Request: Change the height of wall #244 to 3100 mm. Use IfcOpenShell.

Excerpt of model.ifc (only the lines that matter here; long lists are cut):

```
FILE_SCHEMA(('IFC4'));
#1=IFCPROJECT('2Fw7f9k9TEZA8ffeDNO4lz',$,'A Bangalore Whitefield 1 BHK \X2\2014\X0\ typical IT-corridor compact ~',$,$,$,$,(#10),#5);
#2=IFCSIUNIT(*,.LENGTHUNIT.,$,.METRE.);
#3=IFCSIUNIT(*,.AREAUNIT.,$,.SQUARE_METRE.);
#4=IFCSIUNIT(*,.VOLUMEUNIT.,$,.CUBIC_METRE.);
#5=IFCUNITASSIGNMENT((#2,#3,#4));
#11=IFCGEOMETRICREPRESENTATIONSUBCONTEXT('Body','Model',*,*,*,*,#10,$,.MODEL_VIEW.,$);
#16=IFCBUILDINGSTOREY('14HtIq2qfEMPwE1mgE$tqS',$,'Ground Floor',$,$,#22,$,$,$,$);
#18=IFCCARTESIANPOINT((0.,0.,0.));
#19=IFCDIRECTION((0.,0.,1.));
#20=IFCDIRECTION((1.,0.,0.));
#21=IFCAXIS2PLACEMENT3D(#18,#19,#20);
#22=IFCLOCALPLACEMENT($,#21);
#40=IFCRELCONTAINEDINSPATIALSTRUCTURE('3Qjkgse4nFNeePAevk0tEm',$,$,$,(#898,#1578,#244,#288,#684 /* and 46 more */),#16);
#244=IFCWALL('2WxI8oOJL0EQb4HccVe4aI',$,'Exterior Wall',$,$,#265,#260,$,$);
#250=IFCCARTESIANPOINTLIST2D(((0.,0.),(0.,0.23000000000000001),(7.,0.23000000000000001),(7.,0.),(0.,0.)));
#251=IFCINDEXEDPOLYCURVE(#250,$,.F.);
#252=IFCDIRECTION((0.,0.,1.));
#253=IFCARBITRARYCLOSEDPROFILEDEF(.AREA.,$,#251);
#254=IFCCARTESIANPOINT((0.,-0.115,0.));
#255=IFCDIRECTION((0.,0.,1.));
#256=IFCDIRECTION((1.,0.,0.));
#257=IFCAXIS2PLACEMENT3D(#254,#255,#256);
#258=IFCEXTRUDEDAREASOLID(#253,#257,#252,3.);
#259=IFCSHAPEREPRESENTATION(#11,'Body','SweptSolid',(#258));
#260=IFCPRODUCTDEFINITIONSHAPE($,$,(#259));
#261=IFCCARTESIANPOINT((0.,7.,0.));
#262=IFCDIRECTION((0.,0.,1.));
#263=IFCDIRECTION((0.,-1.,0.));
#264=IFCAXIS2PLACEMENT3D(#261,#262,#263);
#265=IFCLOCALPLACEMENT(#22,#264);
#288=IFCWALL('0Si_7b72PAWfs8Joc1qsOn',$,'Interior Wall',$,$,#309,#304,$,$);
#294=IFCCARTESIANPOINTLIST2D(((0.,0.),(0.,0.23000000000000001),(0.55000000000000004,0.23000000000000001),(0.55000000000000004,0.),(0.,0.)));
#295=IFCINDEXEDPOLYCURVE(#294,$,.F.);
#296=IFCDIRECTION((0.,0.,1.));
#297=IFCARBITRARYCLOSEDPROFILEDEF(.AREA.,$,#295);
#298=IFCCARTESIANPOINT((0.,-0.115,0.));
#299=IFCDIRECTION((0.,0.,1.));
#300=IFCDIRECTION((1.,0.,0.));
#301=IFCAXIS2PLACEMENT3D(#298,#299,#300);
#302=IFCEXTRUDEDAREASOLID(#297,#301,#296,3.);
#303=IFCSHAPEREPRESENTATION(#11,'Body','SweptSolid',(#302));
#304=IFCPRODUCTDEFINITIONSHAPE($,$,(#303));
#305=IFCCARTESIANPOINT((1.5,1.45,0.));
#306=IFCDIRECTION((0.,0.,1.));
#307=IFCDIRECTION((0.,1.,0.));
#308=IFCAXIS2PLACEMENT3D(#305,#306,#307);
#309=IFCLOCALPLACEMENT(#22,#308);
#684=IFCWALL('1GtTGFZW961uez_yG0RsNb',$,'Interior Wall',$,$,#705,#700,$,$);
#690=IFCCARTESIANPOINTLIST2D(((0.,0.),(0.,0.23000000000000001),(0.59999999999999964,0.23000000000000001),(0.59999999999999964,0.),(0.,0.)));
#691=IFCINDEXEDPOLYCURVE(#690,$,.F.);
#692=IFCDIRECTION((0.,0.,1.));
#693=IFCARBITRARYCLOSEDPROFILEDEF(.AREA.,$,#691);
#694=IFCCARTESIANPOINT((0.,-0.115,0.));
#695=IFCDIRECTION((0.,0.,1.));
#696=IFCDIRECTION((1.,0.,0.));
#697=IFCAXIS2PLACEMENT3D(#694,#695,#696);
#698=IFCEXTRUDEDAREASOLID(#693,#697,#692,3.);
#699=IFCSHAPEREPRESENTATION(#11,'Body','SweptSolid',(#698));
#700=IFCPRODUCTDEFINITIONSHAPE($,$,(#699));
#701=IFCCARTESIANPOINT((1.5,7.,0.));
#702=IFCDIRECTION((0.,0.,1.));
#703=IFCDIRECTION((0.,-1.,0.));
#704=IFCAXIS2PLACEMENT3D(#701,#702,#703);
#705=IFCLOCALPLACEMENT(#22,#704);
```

```python
import ifcopenshell
import ifcopenshell.geom
import ifcopenshell.util.representation
import ifcopenshell.util.shape
import ifcopenshell.util.unit

model = ifcopenshell.open("model.ifc")
unit_scale = ifcopenshell.util.unit.calculate_unit_scale(model)
settings = ifcopenshell.geom.settings()


def volume(element):
    """Net volume in cubic metres, openings subtracted."""
    shape = ifcopenshell.geom.create_shape(settings, element)
    return ifcopenshell.util.shape.get_volume(shape.geometry)


wall = model.by_guid("2WxI8oOJL0EQb4HccVe4aI")
before = volume(wall)

body = ifcopenshell.util.representation.get_representation(wall, "Model", "Body")
solid = body.Items[0]
old_height = solid.Depth
solid.Depth = 3.1 / unit_scale
after = volume(wall)

print(f"height {old_height:g} -> {solid.Depth:g}, volume {before:.3f} -> {after:.3f} m3")

model.write("model-out.ifc")
```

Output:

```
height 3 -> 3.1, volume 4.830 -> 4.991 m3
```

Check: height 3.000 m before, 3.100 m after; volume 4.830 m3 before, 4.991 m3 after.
